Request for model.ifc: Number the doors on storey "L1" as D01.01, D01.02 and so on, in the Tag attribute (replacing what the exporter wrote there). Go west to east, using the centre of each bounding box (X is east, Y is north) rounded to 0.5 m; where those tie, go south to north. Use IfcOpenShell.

First a look at what the model holds.

```python
import ifcopenshell
import ifcopenshell.util.element
import ifcopenshell.util.placement

model = ifcopenshell.open("model.ifc")
print(model.schema)
storey = next(s for s in model.by_type("IfcBuildingStorey") if s.Name == "L1")
doors = [e for e in ifcopenshell.util.element.get_decomposition(storey) if e.is_a("IfcDoor")]
for e in sorted(doors, key=lambda e: e.id()):
    origin = ifcopenshell.util.placement.get_local_placement(e.ObjectPlacement)[:3, 3]
    print(e.id(), e.Tag, e.Name, origin.round(2) + 0.0, sep=" | ")
```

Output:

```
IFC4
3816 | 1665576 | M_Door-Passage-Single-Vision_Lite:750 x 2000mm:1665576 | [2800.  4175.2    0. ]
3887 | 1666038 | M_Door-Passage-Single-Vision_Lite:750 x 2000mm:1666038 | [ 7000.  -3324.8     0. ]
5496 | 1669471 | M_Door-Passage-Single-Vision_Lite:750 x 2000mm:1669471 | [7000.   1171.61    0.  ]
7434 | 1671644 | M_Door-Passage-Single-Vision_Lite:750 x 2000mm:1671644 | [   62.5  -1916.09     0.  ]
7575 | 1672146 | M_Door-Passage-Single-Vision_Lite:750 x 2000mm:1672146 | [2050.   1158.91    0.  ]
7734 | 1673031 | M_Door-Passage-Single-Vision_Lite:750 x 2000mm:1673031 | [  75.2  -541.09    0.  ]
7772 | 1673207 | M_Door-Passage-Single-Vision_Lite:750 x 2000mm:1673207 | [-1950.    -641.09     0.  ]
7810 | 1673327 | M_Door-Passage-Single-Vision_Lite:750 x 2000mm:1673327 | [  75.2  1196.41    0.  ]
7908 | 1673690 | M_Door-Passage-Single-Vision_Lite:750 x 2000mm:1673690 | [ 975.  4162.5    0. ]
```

```python
import ifcopenshell
import ifcopenshell.geom
import ifcopenshell.util.element
import ifcopenshell.util.shape

model = ifcopenshell.open("model.ifc")
settings = ifcopenshell.geom.settings()
settings.set("use-world-coords", True)


def centre(element):
    shape = ifcopenshell.geom.create_shape(settings, element)
    return ifcopenshell.util.shape.get_bbox_centroid(shape.geometry)


storey = next(s for s in model.by_type("IfcBuildingStorey") if s.Name == "L1")
doors = [e for e in ifcopenshell.util.element.get_decomposition(storey) if e.is_a("IfcDoor")]

# Insertion points can sit at a corner or the storey origin, so sort by the geometry (in metres).
centres = {e: centre(e) for e in doors}
doors.sort(key=lambda e: (round(centres[e][0] / 0.5), centres[e][1]))

for i, e in enumerate(doors, start=1):
    number = f"D01.{i:02d}"
    e.Tag = number
    print(e.id(), number)

model.write("model_rev.ifc")
```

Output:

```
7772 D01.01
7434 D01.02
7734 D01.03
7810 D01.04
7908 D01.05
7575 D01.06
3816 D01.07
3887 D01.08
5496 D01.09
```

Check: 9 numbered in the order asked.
